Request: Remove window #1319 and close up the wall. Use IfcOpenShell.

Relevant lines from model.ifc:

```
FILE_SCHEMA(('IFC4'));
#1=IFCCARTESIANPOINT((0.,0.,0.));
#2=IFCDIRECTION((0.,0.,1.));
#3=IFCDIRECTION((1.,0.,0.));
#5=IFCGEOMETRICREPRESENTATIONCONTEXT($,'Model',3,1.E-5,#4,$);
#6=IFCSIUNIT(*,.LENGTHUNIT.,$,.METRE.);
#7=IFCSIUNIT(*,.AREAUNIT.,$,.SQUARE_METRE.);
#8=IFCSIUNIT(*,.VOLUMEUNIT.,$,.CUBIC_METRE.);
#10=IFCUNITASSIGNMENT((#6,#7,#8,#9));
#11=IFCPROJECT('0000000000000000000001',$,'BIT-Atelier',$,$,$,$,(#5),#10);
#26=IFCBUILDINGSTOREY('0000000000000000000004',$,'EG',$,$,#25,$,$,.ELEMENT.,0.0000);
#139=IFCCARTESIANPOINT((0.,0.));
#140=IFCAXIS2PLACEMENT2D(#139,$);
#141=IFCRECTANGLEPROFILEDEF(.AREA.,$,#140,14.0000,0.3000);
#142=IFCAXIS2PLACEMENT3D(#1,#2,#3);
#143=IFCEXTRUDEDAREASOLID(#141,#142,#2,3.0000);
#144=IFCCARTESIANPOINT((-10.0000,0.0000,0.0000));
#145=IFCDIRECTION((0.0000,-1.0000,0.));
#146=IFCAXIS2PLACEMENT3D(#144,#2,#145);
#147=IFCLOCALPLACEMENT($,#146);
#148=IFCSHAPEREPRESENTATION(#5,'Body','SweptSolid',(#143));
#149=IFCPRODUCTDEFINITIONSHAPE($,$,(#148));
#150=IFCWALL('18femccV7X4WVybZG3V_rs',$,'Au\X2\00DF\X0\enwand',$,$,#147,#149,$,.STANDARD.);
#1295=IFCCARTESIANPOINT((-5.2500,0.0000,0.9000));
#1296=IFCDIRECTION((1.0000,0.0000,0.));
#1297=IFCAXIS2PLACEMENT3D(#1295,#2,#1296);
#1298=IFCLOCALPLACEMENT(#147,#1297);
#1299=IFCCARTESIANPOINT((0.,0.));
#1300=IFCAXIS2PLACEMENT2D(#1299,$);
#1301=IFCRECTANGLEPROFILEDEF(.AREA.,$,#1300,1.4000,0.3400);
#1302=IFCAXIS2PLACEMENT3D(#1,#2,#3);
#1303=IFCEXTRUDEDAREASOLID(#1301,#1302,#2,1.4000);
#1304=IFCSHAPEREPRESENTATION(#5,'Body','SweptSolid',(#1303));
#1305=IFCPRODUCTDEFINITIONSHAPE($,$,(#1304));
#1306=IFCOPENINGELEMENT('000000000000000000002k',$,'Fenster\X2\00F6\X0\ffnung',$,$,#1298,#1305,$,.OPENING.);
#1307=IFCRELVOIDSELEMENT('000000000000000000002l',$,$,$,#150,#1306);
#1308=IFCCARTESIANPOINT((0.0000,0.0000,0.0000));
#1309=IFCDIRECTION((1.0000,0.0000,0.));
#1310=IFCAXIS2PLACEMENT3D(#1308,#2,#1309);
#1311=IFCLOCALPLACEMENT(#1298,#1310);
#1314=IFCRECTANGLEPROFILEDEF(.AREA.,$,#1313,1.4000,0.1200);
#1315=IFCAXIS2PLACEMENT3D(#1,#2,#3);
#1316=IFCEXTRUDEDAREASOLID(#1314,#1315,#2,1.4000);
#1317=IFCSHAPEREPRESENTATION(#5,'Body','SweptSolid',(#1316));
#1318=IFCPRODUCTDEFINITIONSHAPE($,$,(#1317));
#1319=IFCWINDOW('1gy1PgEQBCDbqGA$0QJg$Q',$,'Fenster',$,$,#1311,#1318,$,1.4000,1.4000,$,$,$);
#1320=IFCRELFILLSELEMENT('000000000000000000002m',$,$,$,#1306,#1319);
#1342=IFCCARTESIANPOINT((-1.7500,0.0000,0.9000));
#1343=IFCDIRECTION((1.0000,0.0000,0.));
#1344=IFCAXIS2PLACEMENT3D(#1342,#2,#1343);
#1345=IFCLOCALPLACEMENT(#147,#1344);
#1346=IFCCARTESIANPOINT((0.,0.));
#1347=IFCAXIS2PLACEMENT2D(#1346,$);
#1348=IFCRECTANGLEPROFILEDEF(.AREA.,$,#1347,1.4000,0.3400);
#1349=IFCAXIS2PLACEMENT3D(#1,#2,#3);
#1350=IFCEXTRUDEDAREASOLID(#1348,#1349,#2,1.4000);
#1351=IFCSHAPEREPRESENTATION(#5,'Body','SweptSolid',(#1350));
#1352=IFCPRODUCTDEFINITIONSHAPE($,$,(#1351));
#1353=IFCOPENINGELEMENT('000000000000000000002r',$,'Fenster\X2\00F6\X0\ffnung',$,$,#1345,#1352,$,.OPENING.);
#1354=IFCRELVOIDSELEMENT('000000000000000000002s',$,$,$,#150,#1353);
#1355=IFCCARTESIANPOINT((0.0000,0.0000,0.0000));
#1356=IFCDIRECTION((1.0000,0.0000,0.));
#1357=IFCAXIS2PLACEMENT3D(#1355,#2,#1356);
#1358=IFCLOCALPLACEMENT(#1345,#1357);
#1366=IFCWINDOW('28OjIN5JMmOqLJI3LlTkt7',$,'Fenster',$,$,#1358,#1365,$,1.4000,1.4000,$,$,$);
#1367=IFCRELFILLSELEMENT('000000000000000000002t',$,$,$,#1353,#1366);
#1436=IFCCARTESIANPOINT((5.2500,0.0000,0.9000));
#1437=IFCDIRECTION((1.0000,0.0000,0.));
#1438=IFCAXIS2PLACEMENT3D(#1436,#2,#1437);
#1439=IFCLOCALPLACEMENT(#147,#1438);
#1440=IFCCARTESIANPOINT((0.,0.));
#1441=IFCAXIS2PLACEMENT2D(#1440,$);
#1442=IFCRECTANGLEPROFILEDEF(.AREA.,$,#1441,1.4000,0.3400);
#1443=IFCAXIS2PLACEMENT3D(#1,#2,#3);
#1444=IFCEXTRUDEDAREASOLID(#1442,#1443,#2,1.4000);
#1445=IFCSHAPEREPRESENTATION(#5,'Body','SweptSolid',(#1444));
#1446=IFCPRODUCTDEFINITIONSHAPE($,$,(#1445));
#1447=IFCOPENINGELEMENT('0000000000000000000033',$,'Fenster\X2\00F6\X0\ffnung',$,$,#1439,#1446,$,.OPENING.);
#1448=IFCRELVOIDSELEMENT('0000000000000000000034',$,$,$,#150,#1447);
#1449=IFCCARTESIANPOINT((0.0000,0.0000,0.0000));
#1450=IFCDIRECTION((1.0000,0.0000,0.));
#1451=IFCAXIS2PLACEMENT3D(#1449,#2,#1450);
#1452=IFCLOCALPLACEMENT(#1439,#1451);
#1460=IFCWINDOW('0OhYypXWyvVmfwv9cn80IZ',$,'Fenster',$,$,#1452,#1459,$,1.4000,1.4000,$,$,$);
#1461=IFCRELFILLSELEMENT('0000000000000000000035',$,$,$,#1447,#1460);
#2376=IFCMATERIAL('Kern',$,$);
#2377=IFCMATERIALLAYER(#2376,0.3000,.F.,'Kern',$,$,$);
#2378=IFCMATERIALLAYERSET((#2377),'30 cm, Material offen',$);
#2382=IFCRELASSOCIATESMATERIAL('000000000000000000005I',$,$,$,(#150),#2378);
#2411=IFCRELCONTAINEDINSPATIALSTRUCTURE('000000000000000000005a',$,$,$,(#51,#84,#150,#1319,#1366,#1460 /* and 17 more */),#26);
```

```python
import ifcopenshell
import ifcopenshell.api.feature
import ifcopenshell.api.root
import ifcopenshell.geom
import ifcopenshell.util.shape

model = ifcopenshell.open("model.ifc")
settings = ifcopenshell.geom.settings()


def volume(element):
    """Net volume in cubic metres, openings subtracted."""
    shape = ifcopenshell.geom.create_shape(settings, element)
    return ifcopenshell.util.shape.get_volume(shape.geometry)


window = model.by_guid("1gy1PgEQBCDbqGA$0QJg$Q")
opening = window.FillsVoids[0].RelatingOpeningElement
wall = opening.VoidsElements[0].RelatingBuildingElement
before = volume(wall)

ifcopenshell.api.root.remove_product(model, product=window)
ifcopenshell.api.feature.remove_feature(model, feature=opening)

after = volume(wall)

print(f"wall volume {before:.3f} -> {after:.3f} m3")

model.write("model_rev.ifc")
```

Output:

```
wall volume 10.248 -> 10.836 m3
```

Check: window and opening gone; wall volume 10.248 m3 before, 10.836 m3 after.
